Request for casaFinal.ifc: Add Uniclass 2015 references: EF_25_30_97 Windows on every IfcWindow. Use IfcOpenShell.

First a look at what the model holds.

```python
import ifcopenshell

model = ifcopenshell.open("casaFinal.ifc")
print(model.schema)
print("classifications:", [c.Name for c in model.by_type("IfcClassification")])
for ifc_class in ("IfcDoor", "IfcRoof", "IfcStair", "IfcWall", "IfcWindow"):
    print(ifc_class, len(model.by_type(ifc_class)))
```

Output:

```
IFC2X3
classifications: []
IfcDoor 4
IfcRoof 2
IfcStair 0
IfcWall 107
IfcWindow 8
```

```python
import ifcopenshell
import ifcopenshell.api.classification

model = ifcopenshell.open("casaFinal.ifc")

# IFC2X3 requires Source and Edition and has no link from the project to the system.
system = model.create_entity("IfcClassification", Source="NBS", Edition="2015", Name="Uniclass 2015")

codes = {
    "IfcWindow": ("EF_25_30_97", "Windows"),
}
for ifc_class, (code, name) in codes.items():
    products = model.by_type(ifc_class)
    ifcopenshell.api.classification.add_reference(
        model, products=products, classification=system, identification=code, name=name
    )
    print(code, len(products))

model.write("casaFinal_rev.ifc")
```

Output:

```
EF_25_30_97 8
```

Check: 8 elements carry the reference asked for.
